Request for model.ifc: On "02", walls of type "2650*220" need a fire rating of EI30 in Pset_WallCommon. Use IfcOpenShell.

First a look at what the model holds.

```python
import ifcopenshell
import ifcopenshell.util.element

model = ifcopenshell.open("model.ifc")
print(model.schema)
storey = next(s for s in model.by_type("IfcBuildingStorey") if s.Name == "02")
walls = [e for e in ifcopenshell.util.element.get_decomposition(storey) if e.is_a("IfcWall")]
seen = {}
for e in walls:
    element_type = ifcopenshell.util.element.get_type(e)
    key = (element_type.Name if element_type != e and element_type else None, ifcopenshell.util.element.get_pset(e, "Pset_WallCommon", "FireRating"))
    seen[key] = seen.get(key, 0) + 1
for (name, value), count in sorted(seen.items(), key=str):
    print(count, "x", name, "|", value)
```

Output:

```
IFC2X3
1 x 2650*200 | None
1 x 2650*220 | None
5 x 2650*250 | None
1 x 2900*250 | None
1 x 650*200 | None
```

```python
import ifcopenshell
import ifcopenshell.api.pset
import ifcopenshell.util.element

model = ifcopenshell.open("model.ifc")

storey = next(s for s in model.by_type("IfcBuildingStorey") if s.Name == "02")
walls = [e for e in ifcopenshell.util.element.get_decomposition(storey) if e.is_a("IfcWall")]

count = 0
for e in walls:
    element_type = ifcopenshell.util.element.get_type(e)
    if element_type in (None, e) or element_type.Name != "2650*220":
        continue
    # add_pset returns the element's existing set when there is one.
    pset = ifcopenshell.api.pset.add_pset(model, product=e, name="Pset_WallCommon")
    ifcopenshell.api.pset.edit_pset(model, pset=pset, properties={"FireRating": "EI30"})
    count += 1

print(count, "walls updated")

model.write("model_v2.ifc")
```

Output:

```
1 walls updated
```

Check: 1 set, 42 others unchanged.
